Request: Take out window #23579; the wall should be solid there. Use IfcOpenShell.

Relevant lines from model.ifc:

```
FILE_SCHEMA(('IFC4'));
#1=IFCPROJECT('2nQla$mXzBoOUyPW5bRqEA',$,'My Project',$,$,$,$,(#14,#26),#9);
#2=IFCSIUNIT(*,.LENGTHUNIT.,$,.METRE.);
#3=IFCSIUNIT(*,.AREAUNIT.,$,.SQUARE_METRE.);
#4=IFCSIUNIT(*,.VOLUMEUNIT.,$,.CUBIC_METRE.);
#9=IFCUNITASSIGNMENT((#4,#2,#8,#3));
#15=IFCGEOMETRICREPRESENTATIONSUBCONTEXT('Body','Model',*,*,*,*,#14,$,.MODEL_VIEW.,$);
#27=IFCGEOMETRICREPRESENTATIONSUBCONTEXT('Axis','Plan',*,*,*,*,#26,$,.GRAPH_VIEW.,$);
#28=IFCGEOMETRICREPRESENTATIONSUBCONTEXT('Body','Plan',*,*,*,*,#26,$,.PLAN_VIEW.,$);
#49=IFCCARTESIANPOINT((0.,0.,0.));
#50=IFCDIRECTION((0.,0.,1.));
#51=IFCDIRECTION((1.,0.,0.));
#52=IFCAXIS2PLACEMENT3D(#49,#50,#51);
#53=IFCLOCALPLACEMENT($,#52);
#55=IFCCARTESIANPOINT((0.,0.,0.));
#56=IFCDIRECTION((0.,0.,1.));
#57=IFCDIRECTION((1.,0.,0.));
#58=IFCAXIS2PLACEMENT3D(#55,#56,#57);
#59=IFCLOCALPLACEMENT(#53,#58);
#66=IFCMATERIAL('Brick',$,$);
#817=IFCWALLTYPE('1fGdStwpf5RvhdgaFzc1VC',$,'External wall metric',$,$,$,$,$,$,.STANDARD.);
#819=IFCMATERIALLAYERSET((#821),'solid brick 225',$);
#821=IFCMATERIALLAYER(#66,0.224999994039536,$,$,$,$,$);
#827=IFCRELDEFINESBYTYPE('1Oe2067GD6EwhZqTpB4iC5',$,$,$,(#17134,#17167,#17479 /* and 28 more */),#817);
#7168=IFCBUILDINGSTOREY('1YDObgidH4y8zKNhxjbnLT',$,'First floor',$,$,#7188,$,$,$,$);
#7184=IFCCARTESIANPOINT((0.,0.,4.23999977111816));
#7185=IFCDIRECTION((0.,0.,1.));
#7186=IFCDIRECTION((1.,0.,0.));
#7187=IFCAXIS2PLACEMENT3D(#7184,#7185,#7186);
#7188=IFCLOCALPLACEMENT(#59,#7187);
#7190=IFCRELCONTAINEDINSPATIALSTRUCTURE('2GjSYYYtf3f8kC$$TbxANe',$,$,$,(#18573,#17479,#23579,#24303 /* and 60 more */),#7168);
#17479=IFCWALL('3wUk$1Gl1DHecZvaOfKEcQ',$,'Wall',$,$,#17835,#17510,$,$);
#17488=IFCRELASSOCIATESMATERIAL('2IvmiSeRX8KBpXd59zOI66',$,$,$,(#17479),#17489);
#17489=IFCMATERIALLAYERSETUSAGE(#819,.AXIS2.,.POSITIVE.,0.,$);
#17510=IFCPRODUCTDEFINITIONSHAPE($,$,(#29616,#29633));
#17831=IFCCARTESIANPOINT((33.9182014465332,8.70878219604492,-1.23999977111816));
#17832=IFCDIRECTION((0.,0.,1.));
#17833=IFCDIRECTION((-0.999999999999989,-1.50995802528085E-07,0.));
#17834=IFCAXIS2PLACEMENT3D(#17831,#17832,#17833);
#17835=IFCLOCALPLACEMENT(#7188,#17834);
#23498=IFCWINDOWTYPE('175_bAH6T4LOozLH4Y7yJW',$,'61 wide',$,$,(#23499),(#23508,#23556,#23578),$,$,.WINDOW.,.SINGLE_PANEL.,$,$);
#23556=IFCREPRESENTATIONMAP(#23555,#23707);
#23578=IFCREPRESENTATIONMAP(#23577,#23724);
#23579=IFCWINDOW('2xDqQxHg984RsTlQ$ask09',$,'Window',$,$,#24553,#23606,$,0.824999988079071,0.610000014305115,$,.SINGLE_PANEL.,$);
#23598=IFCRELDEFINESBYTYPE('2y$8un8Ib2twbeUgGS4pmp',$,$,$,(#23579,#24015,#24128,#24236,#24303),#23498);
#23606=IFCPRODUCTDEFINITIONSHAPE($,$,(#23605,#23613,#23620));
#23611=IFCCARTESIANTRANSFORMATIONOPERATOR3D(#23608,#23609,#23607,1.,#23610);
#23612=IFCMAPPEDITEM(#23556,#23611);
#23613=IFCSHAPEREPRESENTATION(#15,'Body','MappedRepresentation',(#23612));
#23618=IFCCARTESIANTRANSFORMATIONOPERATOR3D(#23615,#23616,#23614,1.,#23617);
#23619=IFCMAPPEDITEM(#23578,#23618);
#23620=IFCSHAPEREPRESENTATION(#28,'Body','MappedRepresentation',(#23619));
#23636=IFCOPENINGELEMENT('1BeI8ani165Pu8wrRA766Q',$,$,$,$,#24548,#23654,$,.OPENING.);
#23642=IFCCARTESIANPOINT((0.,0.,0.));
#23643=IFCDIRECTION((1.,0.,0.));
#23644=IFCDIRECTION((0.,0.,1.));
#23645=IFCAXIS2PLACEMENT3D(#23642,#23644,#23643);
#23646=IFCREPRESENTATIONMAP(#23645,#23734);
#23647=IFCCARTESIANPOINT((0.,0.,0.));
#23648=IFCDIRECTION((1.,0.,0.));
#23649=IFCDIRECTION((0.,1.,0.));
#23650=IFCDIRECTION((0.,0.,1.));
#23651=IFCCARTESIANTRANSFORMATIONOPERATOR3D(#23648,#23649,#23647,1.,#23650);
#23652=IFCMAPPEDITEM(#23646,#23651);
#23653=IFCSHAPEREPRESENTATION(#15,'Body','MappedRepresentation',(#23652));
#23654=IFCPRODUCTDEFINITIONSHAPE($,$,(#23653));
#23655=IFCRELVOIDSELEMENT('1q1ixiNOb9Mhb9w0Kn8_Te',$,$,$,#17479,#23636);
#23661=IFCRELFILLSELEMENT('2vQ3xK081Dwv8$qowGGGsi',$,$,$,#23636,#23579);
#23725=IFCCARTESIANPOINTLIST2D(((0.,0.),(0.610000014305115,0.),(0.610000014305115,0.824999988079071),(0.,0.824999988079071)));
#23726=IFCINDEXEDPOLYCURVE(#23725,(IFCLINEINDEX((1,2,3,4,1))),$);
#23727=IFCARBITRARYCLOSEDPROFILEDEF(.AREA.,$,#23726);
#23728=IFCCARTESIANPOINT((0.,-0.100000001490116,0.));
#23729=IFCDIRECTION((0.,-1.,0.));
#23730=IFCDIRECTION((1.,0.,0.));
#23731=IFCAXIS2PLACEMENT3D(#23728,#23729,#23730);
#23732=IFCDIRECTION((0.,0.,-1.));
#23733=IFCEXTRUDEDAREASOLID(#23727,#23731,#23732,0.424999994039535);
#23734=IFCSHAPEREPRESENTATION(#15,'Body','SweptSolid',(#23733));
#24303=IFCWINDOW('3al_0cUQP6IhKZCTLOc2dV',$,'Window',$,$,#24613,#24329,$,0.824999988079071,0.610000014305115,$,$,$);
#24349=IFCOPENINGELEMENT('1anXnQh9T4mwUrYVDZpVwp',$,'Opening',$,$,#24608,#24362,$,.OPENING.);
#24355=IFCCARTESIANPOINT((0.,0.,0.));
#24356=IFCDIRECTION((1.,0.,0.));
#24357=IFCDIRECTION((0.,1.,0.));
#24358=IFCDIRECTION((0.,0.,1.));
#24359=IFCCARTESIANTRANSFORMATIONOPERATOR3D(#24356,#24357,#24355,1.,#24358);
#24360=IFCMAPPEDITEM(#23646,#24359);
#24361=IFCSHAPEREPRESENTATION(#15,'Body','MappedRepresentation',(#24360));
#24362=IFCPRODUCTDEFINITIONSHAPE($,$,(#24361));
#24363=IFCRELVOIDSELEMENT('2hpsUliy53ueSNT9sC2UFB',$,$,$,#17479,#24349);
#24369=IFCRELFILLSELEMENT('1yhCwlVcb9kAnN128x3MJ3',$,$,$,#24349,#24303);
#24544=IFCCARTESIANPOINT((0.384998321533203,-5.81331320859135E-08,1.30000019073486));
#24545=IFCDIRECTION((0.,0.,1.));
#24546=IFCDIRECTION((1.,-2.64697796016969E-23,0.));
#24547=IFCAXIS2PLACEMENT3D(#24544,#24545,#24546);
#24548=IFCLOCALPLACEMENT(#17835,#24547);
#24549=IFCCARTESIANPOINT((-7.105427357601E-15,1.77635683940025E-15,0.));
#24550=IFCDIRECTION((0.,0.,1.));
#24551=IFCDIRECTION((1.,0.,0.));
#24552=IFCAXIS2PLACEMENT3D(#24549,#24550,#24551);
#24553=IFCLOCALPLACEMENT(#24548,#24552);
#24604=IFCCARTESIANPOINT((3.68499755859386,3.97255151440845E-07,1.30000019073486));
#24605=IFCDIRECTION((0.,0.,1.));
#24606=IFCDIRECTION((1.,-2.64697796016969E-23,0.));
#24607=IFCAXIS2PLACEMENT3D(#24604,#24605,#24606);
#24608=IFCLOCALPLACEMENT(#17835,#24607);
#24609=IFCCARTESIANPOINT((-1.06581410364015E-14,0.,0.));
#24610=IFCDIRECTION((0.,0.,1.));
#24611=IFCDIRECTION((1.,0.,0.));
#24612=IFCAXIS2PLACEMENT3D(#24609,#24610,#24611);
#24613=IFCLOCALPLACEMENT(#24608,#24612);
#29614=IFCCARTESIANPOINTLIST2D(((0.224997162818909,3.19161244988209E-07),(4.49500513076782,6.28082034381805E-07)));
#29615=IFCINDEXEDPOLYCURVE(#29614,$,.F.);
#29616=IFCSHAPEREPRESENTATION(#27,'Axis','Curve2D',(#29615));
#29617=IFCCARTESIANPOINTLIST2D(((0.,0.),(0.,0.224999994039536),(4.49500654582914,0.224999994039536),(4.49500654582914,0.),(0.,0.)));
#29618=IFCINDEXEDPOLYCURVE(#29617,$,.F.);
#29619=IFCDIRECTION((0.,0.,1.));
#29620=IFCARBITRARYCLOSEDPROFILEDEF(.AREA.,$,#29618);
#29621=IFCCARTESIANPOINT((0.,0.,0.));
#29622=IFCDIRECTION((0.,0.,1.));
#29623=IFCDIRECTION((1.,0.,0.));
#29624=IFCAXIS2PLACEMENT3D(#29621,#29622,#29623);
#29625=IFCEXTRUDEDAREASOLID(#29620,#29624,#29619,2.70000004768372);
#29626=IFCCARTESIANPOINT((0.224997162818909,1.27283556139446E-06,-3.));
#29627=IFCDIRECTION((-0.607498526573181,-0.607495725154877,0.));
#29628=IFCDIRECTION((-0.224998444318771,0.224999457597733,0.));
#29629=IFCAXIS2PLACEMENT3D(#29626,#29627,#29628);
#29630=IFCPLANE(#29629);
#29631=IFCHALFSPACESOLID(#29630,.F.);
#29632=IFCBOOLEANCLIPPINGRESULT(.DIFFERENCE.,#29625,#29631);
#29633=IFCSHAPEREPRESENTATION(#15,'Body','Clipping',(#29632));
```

```python
import ifcopenshell
import ifcopenshell.api.feature
import ifcopenshell.api.root
import ifcopenshell.geom
import ifcopenshell.util.shape

model = ifcopenshell.open("model.ifc")
settings = ifcopenshell.geom.settings()


def volume(element):
    """Net volume in cubic metres, openings subtracted."""
    shape = ifcopenshell.geom.create_shape(settings, element)
    return ifcopenshell.util.shape.get_volume(shape.geometry)


window = model.by_guid("2xDqQxHg984RsTlQ$ask09")
opening = window.FillsVoids[0].RelatingOpeningElement
wall = opening.VoidsElements[0].RelatingBuildingElement
before = volume(wall)

ifcopenshell.api.root.remove_product(model, product=window)
ifcopenshell.api.feature.remove_feature(model, feature=opening)

after = volume(wall)

print(f"wall volume {before:.3f} -> {after:.3f} m3")

model.write("model_rev.ifc")
```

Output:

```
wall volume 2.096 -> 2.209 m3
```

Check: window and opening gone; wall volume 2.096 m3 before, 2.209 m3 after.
